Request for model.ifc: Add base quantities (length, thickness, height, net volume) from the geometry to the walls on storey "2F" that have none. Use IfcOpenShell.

First a look at what the model holds.

```python
import ifcopenshell
import ifcopenshell.util.element
import ifcopenshell.util.unit

model = ifcopenshell.open("model.ifc")
print(model.schema)
for unit_type in ("LENGTHUNIT", "AREAUNIT", "VOLUMEUNIT"):
    print(unit_type, ifcopenshell.util.unit.calculate_unit_scale(model, unit_type))
storey = next(s for s in model.by_type("IfcBuildingStorey") if s.Name == "2F")
walls = [e for e in ifcopenshell.util.element.get_decomposition(storey) if e.is_a("IfcWall")]
for e in sorted(walls, key=lambda e: e.id()):
    print(e.id(), e.is_a(), e.Name, list(ifcopenshell.util.element.get_psets(e, qtos_only=True)), sep=" | ")
```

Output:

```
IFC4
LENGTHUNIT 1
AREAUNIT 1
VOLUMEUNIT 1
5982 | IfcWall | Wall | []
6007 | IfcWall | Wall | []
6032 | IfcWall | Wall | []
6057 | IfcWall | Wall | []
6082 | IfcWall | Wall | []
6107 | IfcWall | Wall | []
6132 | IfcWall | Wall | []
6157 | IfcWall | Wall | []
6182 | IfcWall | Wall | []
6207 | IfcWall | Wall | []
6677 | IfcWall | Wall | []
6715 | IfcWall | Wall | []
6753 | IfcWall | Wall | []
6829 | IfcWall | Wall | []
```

```python
import ifcopenshell
import ifcopenshell.api.pset
import ifcopenshell.geom
import ifcopenshell.util.element
import ifcopenshell.util.shape
import ifcopenshell.util.unit

model = ifcopenshell.open("model.ifc")
unit_scale = ifcopenshell.util.unit.calculate_unit_scale(model)
volume_scale = ifcopenshell.util.unit.calculate_unit_scale(model, "VOLUMEUNIT")
settings = ifcopenshell.geom.settings()

storey = next(s for s in model.by_type("IfcBuildingStorey") if s.Name == "2F")
walls = [e for e in ifcopenshell.util.element.get_decomposition(storey) if e.is_a("IfcWall")]

for e in sorted(walls, key=lambda e: e.id()):
    if ifcopenshell.util.element.get_psets(e, qtos_only=True, should_inherit=False):
        continue
    # Geometry comes back in metres, in the element's own axes.
    shape = ifcopenshell.geom.create_shape(settings, e)
    values = {
        "Length": ifcopenshell.util.shape.get_x(shape.geometry) / unit_scale,
        "Width": ifcopenshell.util.shape.get_y(shape.geometry) / unit_scale,
        "Height": ifcopenshell.util.shape.get_z(shape.geometry) / unit_scale,
        "NetVolume": ifcopenshell.util.shape.get_volume(shape.geometry) / volume_scale,
    }
    qto = ifcopenshell.api.pset.add_qto(model, product=e, name="Qto_WallBaseQuantities")
    ifcopenshell.api.pset.edit_qto(model, qto=qto, properties=values)
    print(e.id(), {k: round(v, 3) for k, v in values.items()})

model.write("model_v2.ifc")
```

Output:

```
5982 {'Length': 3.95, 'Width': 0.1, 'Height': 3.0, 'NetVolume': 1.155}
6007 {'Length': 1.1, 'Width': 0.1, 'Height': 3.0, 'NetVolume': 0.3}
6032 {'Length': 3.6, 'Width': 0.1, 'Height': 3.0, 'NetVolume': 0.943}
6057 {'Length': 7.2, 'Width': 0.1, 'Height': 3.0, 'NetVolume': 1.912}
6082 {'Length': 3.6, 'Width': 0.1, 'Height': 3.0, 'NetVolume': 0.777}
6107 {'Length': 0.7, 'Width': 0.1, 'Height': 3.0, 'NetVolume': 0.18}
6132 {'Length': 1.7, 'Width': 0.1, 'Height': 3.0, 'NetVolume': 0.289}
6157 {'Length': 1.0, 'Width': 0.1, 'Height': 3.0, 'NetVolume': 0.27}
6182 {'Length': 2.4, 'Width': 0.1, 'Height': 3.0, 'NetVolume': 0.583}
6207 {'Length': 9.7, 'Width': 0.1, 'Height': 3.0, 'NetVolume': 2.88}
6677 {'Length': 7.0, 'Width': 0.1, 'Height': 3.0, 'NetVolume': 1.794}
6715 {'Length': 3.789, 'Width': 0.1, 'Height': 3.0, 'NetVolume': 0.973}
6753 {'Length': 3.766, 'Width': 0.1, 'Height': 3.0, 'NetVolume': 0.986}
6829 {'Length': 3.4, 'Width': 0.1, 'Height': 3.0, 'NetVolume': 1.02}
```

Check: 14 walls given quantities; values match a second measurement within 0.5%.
